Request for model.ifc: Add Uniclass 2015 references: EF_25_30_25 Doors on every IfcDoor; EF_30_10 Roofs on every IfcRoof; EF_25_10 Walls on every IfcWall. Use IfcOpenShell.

First a look at what the model holds.

```python
import ifcopenshell

model = ifcopenshell.open("model.ifc")
print(model.schema)
print("classifications:", [c.Name for c in model.by_type("IfcClassification")])
for ifc_class in ("IfcDoor", "IfcRoof", "IfcStair", "IfcWall", "IfcWindow"):
    print(ifc_class, len(model.by_type(ifc_class)))
```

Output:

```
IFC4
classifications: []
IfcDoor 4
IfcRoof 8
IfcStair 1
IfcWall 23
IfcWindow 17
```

```python
import ifcopenshell
import ifcopenshell.api.classification

model = ifcopenshell.open("model.ifc")

system = ifcopenshell.api.classification.add_classification(model, classification="Uniclass 2015")

codes = {
    "IfcDoor": ("EF_25_30_25", "Doors"),
    "IfcRoof": ("EF_30_10", "Roofs"),
    "IfcWall": ("EF_25_10", "Walls"),
}
for ifc_class, (code, name) in codes.items():
    products = model.by_type(ifc_class)
    ifcopenshell.api.classification.add_reference(
        model, products=products, classification=system, identification=code, name=name
    )
    print(code, len(products))

model.write("model_updated.ifc")
```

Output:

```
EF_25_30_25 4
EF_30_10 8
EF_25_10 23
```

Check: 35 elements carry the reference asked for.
